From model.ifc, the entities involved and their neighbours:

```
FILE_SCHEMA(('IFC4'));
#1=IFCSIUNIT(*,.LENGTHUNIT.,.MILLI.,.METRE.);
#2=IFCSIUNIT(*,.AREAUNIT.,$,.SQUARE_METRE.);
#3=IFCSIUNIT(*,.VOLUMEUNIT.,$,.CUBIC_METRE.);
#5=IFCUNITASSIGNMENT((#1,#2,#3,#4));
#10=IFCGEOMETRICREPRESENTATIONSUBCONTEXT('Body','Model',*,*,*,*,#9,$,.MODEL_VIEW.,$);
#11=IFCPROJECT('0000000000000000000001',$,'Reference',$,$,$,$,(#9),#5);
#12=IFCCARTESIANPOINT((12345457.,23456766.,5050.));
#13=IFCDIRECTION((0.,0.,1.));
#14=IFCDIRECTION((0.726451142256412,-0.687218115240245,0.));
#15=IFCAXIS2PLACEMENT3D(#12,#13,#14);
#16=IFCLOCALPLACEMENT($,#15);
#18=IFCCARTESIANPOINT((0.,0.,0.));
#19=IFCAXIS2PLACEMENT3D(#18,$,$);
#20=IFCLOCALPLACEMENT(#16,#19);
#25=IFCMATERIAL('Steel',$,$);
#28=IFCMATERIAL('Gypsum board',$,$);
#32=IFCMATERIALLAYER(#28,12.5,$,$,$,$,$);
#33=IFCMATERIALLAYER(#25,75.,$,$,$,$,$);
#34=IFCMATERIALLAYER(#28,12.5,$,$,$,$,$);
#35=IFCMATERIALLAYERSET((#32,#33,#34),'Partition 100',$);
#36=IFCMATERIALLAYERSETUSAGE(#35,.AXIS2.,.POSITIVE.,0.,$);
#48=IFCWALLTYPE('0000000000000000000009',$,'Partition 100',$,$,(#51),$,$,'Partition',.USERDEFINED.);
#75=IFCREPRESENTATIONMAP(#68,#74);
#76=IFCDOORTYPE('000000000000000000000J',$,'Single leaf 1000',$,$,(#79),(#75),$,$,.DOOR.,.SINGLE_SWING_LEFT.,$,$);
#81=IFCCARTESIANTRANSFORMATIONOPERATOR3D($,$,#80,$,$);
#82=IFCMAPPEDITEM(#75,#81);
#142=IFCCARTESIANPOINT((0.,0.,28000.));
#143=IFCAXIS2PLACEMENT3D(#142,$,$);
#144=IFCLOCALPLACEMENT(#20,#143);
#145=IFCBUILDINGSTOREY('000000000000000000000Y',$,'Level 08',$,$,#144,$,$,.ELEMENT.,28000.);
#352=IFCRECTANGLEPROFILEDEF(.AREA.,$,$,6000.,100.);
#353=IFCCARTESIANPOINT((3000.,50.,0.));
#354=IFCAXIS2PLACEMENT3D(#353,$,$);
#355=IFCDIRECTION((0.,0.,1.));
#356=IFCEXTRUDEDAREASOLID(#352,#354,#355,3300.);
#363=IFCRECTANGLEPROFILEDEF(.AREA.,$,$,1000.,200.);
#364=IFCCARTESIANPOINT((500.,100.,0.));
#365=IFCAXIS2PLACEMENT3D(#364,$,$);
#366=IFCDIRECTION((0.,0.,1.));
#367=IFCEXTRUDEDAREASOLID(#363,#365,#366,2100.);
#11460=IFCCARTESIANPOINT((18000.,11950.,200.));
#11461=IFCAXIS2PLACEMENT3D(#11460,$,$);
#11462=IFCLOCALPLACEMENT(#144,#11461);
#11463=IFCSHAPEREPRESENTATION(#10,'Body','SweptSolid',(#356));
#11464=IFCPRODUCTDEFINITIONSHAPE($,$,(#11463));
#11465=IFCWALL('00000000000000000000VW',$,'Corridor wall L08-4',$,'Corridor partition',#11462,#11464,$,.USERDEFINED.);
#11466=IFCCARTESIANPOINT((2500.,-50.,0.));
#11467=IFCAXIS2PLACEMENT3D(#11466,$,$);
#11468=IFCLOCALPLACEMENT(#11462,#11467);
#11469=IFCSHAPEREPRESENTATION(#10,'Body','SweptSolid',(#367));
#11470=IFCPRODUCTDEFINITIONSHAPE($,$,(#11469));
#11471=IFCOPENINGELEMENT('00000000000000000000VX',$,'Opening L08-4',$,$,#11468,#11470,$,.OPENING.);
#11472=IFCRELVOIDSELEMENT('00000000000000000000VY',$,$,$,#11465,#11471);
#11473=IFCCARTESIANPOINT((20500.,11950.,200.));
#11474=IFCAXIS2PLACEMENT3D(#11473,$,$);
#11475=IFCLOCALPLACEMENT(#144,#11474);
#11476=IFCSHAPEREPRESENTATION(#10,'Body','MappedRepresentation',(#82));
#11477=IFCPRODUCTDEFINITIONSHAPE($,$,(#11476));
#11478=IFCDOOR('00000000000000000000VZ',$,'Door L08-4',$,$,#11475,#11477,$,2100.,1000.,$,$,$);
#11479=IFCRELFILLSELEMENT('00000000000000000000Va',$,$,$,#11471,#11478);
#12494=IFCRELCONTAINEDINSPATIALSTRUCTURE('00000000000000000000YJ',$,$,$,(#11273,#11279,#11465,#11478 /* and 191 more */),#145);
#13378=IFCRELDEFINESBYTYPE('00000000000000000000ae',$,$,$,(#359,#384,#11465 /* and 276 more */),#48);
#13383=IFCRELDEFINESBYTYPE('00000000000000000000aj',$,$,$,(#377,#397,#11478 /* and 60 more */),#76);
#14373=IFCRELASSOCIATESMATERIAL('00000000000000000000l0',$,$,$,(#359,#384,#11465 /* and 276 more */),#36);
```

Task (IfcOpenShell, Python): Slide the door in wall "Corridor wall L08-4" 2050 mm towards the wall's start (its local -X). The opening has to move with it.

```python
import ifcopenshell
import ifcopenshell.api.geometry
import ifcopenshell.util.placement
import ifcopenshell.util.unit

model = ifcopenshell.open("model.ifc")
unit_scale = ifcopenshell.util.unit.calculate_unit_scale(model)

door = model.by_guid("00000000000000000000VZ")
opening = door.FillsVoids[0].RelatingOpeningElement
wall = opening.VoidsElements[0].RelatingBuildingElement

wall_matrix = ifcopenshell.util.placement.get_local_placement(wall.ObjectPlacement)
shift = wall_matrix[:3, 0] * -2.05 / unit_scale
before = ifcopenshell.util.placement.get_local_placement(door.ObjectPlacement)[:3, 3].copy()

# The door is not placed relative to its opening, so move both.
for product in (opening, door):
    matrix = ifcopenshell.util.placement.get_local_placement(product.ObjectPlacement)
    matrix[:3, 3] += shift
    ifcopenshell.api.geometry.edit_object_placement(model, product=product, matrix=matrix, is_si=False)

after = ifcopenshell.util.placement.get_local_placement(door.ObjectPlacement)[:3, 3]
print("door moved by", (after - before).round(3) + 0.0)

model.write("model_v2.ifc")
```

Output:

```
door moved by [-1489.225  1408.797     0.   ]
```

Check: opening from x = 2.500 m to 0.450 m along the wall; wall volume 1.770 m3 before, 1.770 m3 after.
